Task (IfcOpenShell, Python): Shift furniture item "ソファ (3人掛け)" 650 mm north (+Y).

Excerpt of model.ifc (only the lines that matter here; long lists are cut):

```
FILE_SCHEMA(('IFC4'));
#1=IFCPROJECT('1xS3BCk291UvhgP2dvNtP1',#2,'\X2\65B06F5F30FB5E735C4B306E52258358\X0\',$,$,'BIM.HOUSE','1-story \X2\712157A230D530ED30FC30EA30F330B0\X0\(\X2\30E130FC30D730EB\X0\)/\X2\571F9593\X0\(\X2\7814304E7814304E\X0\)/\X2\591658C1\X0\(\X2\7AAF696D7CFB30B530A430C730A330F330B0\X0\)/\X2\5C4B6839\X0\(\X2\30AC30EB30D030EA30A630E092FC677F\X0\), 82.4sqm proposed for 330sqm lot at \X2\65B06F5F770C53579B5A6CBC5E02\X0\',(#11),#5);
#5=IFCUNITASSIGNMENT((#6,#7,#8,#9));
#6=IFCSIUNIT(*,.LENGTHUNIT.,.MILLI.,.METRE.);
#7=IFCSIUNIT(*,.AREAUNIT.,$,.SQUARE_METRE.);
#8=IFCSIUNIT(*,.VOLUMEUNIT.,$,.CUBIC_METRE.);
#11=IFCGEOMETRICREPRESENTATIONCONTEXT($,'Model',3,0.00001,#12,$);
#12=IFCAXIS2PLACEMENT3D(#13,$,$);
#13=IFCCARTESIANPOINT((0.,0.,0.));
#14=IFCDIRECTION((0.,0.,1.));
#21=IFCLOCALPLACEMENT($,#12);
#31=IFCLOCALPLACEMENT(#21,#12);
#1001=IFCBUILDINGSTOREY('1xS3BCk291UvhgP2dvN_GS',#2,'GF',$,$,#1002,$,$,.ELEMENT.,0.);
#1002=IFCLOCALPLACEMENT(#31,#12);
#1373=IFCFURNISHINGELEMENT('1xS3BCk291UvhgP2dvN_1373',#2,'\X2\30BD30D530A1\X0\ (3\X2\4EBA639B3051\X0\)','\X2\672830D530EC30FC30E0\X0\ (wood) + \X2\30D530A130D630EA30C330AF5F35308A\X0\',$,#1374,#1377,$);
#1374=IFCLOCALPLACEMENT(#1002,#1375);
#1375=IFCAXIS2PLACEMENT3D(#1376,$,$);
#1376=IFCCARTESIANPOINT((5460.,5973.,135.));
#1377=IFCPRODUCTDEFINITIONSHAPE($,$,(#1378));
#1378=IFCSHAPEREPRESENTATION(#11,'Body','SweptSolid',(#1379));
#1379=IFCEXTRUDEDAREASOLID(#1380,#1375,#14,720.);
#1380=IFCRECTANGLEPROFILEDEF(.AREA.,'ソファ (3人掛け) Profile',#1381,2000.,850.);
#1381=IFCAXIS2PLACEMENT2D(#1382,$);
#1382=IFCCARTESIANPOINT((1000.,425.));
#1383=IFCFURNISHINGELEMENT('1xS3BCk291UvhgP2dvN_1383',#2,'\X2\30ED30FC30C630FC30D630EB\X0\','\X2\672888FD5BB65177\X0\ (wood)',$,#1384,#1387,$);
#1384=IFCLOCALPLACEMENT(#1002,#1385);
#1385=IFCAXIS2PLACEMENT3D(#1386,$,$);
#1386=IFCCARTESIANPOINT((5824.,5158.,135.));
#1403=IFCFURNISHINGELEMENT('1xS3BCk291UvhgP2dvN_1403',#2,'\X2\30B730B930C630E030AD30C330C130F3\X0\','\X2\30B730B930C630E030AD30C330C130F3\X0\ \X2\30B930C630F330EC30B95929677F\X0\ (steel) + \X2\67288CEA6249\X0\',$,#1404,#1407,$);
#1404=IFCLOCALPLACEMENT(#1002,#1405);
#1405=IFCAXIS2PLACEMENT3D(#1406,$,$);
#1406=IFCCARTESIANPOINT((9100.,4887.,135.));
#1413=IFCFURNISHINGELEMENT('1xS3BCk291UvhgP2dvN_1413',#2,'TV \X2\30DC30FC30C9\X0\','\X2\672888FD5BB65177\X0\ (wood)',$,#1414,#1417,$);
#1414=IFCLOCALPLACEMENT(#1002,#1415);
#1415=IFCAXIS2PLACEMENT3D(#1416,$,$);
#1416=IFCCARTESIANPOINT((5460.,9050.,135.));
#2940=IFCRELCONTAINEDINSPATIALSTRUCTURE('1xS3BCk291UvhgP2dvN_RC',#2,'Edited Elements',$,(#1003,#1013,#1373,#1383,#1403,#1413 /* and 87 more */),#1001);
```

```python
import ifcopenshell
import ifcopenshell.api.geometry
import ifcopenshell.util.placement
import ifcopenshell.util.unit

model = ifcopenshell.open("model.ifc")
unit_scale = ifcopenshell.util.unit.calculate_unit_scale(model)

item = model.by_guid("1xS3BCk291UvhgP2dvN_1373")
matrix = ifcopenshell.util.placement.get_local_placement(item.ObjectPlacement)
matrix[1, 3] += 0.65 / unit_scale
ifcopenshell.api.geometry.edit_object_placement(model, product=item, matrix=matrix, is_si=False)

print(ifcopenshell.util.placement.get_local_placement(item.ObjectPlacement).round(3) + 0.0)

model.write("model_edited.ifc")
```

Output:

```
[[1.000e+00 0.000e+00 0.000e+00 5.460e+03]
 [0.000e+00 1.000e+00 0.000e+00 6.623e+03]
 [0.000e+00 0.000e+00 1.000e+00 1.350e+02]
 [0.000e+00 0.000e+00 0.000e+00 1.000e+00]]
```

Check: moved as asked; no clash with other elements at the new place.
